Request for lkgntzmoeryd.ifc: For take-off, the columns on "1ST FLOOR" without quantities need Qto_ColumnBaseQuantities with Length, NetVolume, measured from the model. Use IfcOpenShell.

First a look at what the model holds.

```python
import ifcopenshell
import ifcopenshell.util.element
import ifcopenshell.util.unit

model = ifcopenshell.open("lkgntzmoeryd.ifc")
print(model.schema)
for unit_type in ("LENGTHUNIT", "AREAUNIT", "VOLUMEUNIT"):
    print(unit_type, ifcopenshell.util.unit.calculate_unit_scale(model, unit_type))
storey = next(s for s in model.by_type("IfcBuildingStorey") if s.Name == "1ST FLOOR")
columns = [e for e in ifcopenshell.util.element.get_decomposition(storey) if e.is_a("IfcColumn")]
for e in sorted(columns, key=lambda e: e.id()):
    print(e.id(), e.is_a(), e.Name, list(ifcopenshell.util.element.get_psets(e, qtos_only=True)), sep=" | ")
```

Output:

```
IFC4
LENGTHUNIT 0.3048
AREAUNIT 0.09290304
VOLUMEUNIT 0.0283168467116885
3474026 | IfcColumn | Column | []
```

```python
import ifcopenshell
import ifcopenshell.api.pset
import ifcopenshell.geom
import ifcopenshell.util.element
import ifcopenshell.util.shape
import ifcopenshell.util.unit

model = ifcopenshell.open("lkgntzmoeryd.ifc")
unit_scale = ifcopenshell.util.unit.calculate_unit_scale(model)
volume_scale = ifcopenshell.util.unit.calculate_unit_scale(model, "VOLUMEUNIT")
settings = ifcopenshell.geom.settings()

storey = next(s for s in model.by_type("IfcBuildingStorey") if s.Name == "1ST FLOOR")
columns = [e for e in ifcopenshell.util.element.get_decomposition(storey) if e.is_a("IfcColumn")]

for e in sorted(columns, key=lambda e: e.id()):
    if ifcopenshell.util.element.get_psets(e, qtos_only=True, should_inherit=False):
        continue
    # Geometry comes back in metres, in the element's own axes.
    shape = ifcopenshell.geom.create_shape(settings, e)
    values = {
        "Length": ifcopenshell.util.shape.get_z(shape.geometry) / unit_scale,
        "NetVolume": ifcopenshell.util.shape.get_volume(shape.geometry) / volume_scale,
    }
    qto = ifcopenshell.api.pset.add_qto(model, product=e, name="Qto_ColumnBaseQuantities")
    ifcopenshell.api.pset.edit_qto(model, qto=qto, properties=values)
    print(e.id(), {k: round(v, 3) for k, v in values.items()})

model.write("lkgntzmoeryd-out.ifc")
```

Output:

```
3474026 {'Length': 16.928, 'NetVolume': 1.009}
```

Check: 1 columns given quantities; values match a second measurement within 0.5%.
